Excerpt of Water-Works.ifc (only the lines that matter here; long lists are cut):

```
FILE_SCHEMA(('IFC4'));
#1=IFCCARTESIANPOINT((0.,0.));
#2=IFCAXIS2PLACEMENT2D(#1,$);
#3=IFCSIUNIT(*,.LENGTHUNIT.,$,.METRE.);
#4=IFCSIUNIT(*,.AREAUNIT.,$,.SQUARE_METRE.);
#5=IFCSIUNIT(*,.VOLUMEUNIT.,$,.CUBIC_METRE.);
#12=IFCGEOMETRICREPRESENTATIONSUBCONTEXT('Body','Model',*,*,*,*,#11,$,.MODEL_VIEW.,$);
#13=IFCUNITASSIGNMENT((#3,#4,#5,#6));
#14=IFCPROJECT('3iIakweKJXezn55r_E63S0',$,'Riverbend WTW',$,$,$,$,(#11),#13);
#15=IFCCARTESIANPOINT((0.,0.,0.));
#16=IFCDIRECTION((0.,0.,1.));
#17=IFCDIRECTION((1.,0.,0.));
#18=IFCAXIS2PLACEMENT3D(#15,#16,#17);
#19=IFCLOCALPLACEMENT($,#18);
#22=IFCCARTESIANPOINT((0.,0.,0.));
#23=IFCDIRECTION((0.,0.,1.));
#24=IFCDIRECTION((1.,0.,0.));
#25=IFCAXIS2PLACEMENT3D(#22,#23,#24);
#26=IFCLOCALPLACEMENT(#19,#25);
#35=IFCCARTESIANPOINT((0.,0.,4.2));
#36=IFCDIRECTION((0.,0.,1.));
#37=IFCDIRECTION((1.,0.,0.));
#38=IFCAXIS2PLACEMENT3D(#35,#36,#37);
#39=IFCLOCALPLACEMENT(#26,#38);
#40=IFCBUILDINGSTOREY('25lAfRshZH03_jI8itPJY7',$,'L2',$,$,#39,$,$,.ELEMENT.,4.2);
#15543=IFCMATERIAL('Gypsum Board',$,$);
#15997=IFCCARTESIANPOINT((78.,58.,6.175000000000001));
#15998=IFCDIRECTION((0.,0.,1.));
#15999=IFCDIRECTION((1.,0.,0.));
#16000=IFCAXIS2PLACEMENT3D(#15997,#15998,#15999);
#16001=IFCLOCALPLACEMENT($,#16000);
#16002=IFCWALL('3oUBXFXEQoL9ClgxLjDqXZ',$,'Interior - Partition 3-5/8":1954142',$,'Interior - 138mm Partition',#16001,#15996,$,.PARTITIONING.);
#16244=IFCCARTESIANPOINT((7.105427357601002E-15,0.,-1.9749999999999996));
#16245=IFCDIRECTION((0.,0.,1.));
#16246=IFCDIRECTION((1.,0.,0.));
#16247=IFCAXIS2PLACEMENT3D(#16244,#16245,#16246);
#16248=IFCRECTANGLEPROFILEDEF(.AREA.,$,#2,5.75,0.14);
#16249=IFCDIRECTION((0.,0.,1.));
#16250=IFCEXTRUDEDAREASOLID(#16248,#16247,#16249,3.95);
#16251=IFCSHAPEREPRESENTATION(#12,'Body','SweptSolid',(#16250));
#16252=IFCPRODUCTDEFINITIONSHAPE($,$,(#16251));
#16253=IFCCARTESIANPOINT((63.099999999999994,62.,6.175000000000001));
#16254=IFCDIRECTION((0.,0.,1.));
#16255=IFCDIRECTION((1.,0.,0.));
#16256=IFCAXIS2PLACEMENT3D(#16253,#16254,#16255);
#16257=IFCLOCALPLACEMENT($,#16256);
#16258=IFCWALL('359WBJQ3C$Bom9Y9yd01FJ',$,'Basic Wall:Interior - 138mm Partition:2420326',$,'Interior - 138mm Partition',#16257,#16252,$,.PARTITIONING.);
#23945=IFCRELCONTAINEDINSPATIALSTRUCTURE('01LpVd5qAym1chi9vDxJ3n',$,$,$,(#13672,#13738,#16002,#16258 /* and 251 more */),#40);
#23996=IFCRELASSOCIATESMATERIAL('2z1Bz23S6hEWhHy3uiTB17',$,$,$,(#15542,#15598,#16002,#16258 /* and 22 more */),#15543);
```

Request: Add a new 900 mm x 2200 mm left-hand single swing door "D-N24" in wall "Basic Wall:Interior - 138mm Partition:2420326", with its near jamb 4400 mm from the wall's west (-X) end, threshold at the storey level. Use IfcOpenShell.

```python
import numpy as np
import ifcopenshell
import ifcopenshell.api.feature
import ifcopenshell.api.geometry
import ifcopenshell.api.root
import ifcopenshell.api.spatial
import ifcopenshell.geom
import ifcopenshell.util.element
import ifcopenshell.util.placement
import ifcopenshell.util.representation
import ifcopenshell.util.shape
import ifcopenshell.util.unit

model = ifcopenshell.open("Water-Works.ifc")
unit_scale = ifcopenshell.util.unit.calculate_unit_scale(model)
settings = ifcopenshell.geom.settings()


def volume(element):
    """Net volume in cubic metres, openings subtracted."""
    shape = ifcopenshell.geom.create_shape(settings, element)
    return ifcopenshell.util.shape.get_volume(shape.geometry)


wall = model.by_guid("359WBJQ3C$Bom9Y9yd01FJ")
storey = ifcopenshell.util.element.get_container(wall, ifc_class="IfcBuildingStorey")
context = ifcopenshell.util.representation.get_context(model, "Model", "Body", "MODEL_VIEW")
before = volume(wall)

width, height, from_end, sill = 0.9, 2.2, 4.4, 0.0  # metres

# The wall runs along its own X axis, and the end named is its -X end.
wall_shape = ifcopenshell.geom.create_shape(settings, wall)
x, y, z = ifcopenshell.util.shape.get_vertices(wall_shape.geometry).T
start = x.min() + from_end
face, thickness = float(y.min()), float(y.max() - y.min())
wall_matrix = ifcopenshell.util.placement.get_local_placement(wall.ObjectPlacement)
level = ifcopenshell.util.placement.get_local_placement(storey.ObjectPlacement)[2, 3]


def in_wall(x, y):
    """Placement at x, y metres in the wall's axes, at sill height."""
    matrix = wall_matrix.copy()
    matrix[:, 3] = wall_matrix @ np.array([x / unit_scale, y / unit_scale, 0.0, 1.0])
    matrix[2, 3] = level + sill / unit_scale
    return matrix


# Opening: a box that overshoots both wall faces by 50 mm.
opening = ifcopenshell.api.root.create_entity(model, ifc_class="IfcOpeningElement", predefined_type="OPENING")
box = ifcopenshell.api.geometry.add_wall_representation(
    model, context=context, length=width, height=height, thickness=thickness + 0.1
)
ifcopenshell.api.geometry.assign_representation(model, product=opening, representation=box)
ifcopenshell.api.geometry.edit_object_placement(model, product=opening, matrix=in_wall(start, face - 0.05), is_si=False)
ifcopenshell.api.feature.add_feature(model, feature=opening, element=wall)

door = ifcopenshell.api.root.create_entity(model, ifc_class="IfcDoor", name="D-N24", predefined_type="DOOR")
door.OverallWidth, door.OverallHeight = width / unit_scale, height / unit_scale
door.OperationType = "SINGLE_SWING_LEFT"
body = ifcopenshell.api.geometry.add_door_representation(
    model,
    context=context,
    overall_width=door.OverallWidth,
    overall_height=door.OverallHeight,
    operation_type="SINGLE_SWING_LEFT",
    lining_properties={"LiningDepth": thickness / unit_scale, "ThresholdDepth": thickness / unit_scale},
)
ifcopenshell.api.geometry.assign_representation(model, product=door, representation=body)
ifcopenshell.api.spatial.assign_container(model, products=[door], relating_structure=storey)
ifcopenshell.api.feature.add_filling(model, opening=opening, element=door)

# The lining spans the wall, so the door starts at the wall face.
ifcopenshell.api.geometry.edit_object_placement(model, product=door, matrix=in_wall(start, face), is_si=False)

after = volume(wall)

print(f"wall volume {before:.3f} -> {after:.3f} m3")

model.write("Water-Works_rev.ifc")
```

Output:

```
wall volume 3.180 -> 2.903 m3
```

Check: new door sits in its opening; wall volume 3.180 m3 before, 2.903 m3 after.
